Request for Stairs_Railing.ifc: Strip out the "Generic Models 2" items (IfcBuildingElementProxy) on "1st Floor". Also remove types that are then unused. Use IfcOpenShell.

First a look at what the model holds.

```python
import ifcopenshell
import ifcopenshell.util.element

model = ifcopenshell.open("Stairs_Railing.ifc")
print(model.schema)
storey = next(s for s in model.by_type("IfcBuildingStorey") if s.Name == "1st Floor")
proxies = [e for e in ifcopenshell.util.element.get_decomposition(storey) if e.is_a("IfcBuildingElementProxy")]
seen = {}
for e in proxies:
    element_type = ifcopenshell.util.element.get_type(e)
    name = element_type.Name if element_type not in (None, e) else None
    seen[name] = seen.get(name, 0) + 1
for name, count in sorted(seen.items(), key=str):
    print(count, "x", name)
```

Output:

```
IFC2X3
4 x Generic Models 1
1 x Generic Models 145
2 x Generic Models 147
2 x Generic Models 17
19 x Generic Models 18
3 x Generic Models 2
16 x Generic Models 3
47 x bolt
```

```python
import ifcopenshell
import ifcopenshell.api.root
import ifcopenshell.util.element

model = ifcopenshell.open("Stairs_Railing.ifc")

storey = next(s for s in model.by_type("IfcBuildingStorey") if s.Name == "1st Floor")
proxies = [e for e in ifcopenshell.util.element.get_decomposition(storey) if e.is_a("IfcBuildingElementProxy")]
targets = [e for e in proxies if (t := ifcopenshell.util.element.get_type(e)) not in (None, e) and t.Name == "Generic Models 2"]
types = {ifcopenshell.util.element.get_type(e) for e in targets} - {None, *targets}

for e in targets:
    ifcopenshell.api.root.remove_product(model, product=e)
print(len(targets), "removed")

unused = [t for t in types if not ifcopenshell.util.element.get_types(t)]
for t in unused:
    ifcopenshell.api.root.remove_product(model, product=t)
print(len(unused), "unused types removed")

model.write("Stairs_Railing_updated.ifc")
```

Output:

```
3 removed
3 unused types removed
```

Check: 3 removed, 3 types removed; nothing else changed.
